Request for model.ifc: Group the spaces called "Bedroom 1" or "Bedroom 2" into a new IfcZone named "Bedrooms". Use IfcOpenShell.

First a look at what the model holds.

```python
import ifcopenshell

model = ifcopenshell.open("model.ifc")
print(model.schema)
seen = {}
for space in model.by_type("IfcSpace"):
    seen[space.LongName] = seen.get(space.LongName, 0) + 1
for name, count in sorted(seen.items(), key=str):
    print(count, "x", name)
print("zones:", [z.Name for z in model.by_type("IfcZone")][:20])
```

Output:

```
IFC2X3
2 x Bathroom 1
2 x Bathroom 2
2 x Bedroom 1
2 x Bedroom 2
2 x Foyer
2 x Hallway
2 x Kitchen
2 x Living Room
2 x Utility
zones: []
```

```python
import ifcopenshell
import ifcopenshell.api.group
import ifcopenshell.api.root

model = ifcopenshell.open("model.ifc")

names = {"Bedroom 1", "Bedroom 2"}
spaces = [s for s in model.by_type("IfcSpace") if s.LongName in names]

zone = ifcopenshell.api.root.create_entity(model, ifc_class="IfcZone", name="Bedrooms")
ifcopenshell.api.group.assign_group(model, products=spaces, group=zone)
print(len(spaces), "spaces in", zone.Name)

model.write("model_v2.ifc")
```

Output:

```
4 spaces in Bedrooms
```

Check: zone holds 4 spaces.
